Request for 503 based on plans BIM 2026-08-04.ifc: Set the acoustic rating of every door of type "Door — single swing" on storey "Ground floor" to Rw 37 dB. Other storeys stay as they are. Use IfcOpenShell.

First a look at what the model holds.

```python
import ifcopenshell
import ifcopenshell.util.element

model = ifcopenshell.open("503 based on plans BIM 2026-08-04.ifc")
print(model.schema)
storey = next(s for s in model.by_type("IfcBuildingStorey") if s.Name == "Ground floor")
doors = [e for e in ifcopenshell.util.element.get_decomposition(storey) if e.is_a("IfcDoor")]
seen = {}
for e in doors:
    element_type = ifcopenshell.util.element.get_type(e)
    key = (element_type.Name if element_type != e and element_type else None, ifcopenshell.util.element.get_pset(e, "Pset_DoorCommon", "AcousticRating"))
    seen[key] = seen.get(key, 0) + 1
for (name, value), count in sorted(seen.items(), key=str):
    print(count, "x", name, "|", value)
```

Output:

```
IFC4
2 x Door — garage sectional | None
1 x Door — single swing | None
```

```python
import ifcopenshell
import ifcopenshell.api.pset
import ifcopenshell.util.element

model = ifcopenshell.open("503 based on plans BIM 2026-08-04.ifc")

storey = next(s for s in model.by_type("IfcBuildingStorey") if s.Name == "Ground floor")
doors = [e for e in ifcopenshell.util.element.get_decomposition(storey) if e.is_a("IfcDoor")]

count = 0
for e in doors:
    element_type = ifcopenshell.util.element.get_type(e)
    if element_type in (None, e) or element_type.Name != "Door — single swing":
        continue
    # add_pset returns the element's existing set when there is one.
    pset = ifcopenshell.api.pset.add_pset(model, product=e, name="Pset_DoorCommon")
    ifcopenshell.api.pset.edit_pset(model, pset=pset, properties={"AcousticRating": "Rw 37 dB"})
    count += 1

print(count, "doors updated")

model.write("503 based on plans BIM 2026-08-04_v2.ifc")
```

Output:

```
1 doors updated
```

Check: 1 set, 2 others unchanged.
